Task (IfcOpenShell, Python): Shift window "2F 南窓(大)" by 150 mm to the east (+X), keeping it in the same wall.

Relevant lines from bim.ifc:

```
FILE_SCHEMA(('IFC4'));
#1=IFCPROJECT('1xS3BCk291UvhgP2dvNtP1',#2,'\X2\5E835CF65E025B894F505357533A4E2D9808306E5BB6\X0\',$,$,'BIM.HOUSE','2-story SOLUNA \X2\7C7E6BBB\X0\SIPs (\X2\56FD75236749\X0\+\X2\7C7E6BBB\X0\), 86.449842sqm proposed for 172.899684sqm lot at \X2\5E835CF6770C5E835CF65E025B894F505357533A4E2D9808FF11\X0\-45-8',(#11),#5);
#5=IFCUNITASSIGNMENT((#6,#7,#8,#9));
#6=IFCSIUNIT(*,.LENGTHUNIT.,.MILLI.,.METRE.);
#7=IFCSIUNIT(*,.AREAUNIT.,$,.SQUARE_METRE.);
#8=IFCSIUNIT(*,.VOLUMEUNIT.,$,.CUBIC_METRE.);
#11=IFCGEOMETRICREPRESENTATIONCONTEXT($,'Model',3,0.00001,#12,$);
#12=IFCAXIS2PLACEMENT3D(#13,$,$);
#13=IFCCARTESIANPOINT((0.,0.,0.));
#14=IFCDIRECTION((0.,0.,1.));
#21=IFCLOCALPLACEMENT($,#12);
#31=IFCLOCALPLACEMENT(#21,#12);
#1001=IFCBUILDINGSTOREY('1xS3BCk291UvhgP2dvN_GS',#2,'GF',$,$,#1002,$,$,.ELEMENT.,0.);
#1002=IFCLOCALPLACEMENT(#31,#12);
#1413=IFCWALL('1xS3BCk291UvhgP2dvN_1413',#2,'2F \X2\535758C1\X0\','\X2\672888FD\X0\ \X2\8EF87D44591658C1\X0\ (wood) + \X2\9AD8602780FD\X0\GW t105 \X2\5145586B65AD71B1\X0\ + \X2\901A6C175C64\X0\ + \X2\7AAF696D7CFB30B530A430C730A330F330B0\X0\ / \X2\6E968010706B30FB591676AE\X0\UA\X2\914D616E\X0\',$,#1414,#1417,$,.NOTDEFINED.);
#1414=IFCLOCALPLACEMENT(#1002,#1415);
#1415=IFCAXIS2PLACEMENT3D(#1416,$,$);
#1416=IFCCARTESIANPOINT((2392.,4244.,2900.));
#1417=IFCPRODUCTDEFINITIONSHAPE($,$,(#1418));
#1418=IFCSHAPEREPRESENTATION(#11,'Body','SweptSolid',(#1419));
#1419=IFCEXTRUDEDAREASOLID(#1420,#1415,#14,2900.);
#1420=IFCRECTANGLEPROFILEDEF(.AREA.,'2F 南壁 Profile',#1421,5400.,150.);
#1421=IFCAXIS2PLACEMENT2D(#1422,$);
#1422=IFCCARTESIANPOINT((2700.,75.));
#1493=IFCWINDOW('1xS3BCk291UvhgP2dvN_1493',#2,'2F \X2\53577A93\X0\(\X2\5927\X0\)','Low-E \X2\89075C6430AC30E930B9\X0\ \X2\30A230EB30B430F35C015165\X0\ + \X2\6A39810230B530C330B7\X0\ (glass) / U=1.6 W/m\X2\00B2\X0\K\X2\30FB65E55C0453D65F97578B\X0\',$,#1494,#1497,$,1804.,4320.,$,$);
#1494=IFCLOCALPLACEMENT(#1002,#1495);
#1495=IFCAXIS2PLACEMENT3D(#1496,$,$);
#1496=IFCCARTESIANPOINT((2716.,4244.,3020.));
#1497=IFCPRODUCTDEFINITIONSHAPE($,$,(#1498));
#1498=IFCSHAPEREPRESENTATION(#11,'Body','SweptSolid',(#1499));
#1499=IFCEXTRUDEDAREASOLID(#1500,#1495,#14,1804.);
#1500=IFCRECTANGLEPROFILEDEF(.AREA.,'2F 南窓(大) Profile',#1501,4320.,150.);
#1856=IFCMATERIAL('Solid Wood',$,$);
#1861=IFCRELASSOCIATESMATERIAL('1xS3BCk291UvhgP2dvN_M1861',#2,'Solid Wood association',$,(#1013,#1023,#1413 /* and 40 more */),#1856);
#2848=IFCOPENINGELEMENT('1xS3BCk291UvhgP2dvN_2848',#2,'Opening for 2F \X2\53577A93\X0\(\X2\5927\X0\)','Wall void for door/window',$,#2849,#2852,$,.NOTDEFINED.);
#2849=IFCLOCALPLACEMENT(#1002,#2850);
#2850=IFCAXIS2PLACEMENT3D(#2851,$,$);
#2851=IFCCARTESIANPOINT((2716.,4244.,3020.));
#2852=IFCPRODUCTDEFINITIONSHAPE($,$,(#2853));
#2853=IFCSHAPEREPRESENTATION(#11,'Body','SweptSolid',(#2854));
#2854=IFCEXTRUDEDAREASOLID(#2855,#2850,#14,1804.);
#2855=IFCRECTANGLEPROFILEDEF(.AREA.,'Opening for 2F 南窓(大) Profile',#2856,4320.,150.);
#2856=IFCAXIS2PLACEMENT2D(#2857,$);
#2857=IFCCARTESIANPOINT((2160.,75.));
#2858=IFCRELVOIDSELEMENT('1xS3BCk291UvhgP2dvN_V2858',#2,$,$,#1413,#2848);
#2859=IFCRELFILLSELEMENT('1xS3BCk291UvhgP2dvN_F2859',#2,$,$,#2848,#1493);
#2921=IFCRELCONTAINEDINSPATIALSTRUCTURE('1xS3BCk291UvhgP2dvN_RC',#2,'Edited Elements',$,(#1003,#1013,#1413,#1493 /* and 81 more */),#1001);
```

```python
import ifcopenshell
import ifcopenshell.api.geometry
import ifcopenshell.util.placement
import ifcopenshell.util.unit

model = ifcopenshell.open("bim.ifc")
unit_scale = ifcopenshell.util.unit.calculate_unit_scale(model)

window = model.by_id(1493)
opening = window.FillsVoids[0].RelatingOpeningElement
wall = opening.VoidsElements[0].RelatingBuildingElement

wall_matrix = ifcopenshell.util.placement.get_local_placement(wall.ObjectPlacement)
shift = wall_matrix[:3, 0] * 0.15 / unit_scale
before = ifcopenshell.util.placement.get_local_placement(window.ObjectPlacement)[:3, 3].copy()

# The window is not placed relative to its opening, so move both.
for product in (opening, window):
    matrix = ifcopenshell.util.placement.get_local_placement(product.ObjectPlacement)
    matrix[:3, 3] += shift
    ifcopenshell.api.geometry.edit_object_placement(model, product=product, matrix=matrix, is_si=False)

after = ifcopenshell.util.placement.get_local_placement(window.ObjectPlacement)[:3, 3]
print("window moved by", (after - before).round(3) + 0.0)

model.write("bim_edited.ifc")
```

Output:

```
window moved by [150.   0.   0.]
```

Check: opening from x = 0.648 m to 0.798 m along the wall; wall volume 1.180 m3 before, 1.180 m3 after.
